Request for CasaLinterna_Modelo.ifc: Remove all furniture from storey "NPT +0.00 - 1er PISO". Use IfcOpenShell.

First a look at what the model holds.

```python
import ifcopenshell
import ifcopenshell.util.element

model = ifcopenshell.open("CasaLinterna_Modelo.ifc")
print(model.schema)
storey = next(s for s in model.by_type("IfcBuildingStorey") if s.Name == "NPT +0.00 - 1er PISO")
furniture = [e for e in ifcopenshell.util.element.get_decomposition(storey) if e.is_a("IfcFurnishingElement")]
seen = {}
for e in furniture:
    element_type = ifcopenshell.util.element.get_type(e)
    name = element_type.Name if element_type not in (None, e) else None
    seen[name] = seen.get(name, 0) + 1
for name, count in sorted(seen.items(), key=str):
    print(count, "x", name)
```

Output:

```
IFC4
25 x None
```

```python
import ifcopenshell
import ifcopenshell.api.root
import ifcopenshell.util.element

model = ifcopenshell.open("CasaLinterna_Modelo.ifc")

storey = next(s for s in model.by_type("IfcBuildingStorey") if s.Name == "NPT +0.00 - 1er PISO")
furniture = [e for e in ifcopenshell.util.element.get_decomposition(storey) if e.is_a("IfcFurnishingElement")]

for e in furniture:
    ifcopenshell.api.root.remove_product(model, product=e)
print(len(furniture), "removed")

model.write("CasaLinterna_Modelo_updated.ifc")
```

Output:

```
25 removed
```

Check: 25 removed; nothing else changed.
